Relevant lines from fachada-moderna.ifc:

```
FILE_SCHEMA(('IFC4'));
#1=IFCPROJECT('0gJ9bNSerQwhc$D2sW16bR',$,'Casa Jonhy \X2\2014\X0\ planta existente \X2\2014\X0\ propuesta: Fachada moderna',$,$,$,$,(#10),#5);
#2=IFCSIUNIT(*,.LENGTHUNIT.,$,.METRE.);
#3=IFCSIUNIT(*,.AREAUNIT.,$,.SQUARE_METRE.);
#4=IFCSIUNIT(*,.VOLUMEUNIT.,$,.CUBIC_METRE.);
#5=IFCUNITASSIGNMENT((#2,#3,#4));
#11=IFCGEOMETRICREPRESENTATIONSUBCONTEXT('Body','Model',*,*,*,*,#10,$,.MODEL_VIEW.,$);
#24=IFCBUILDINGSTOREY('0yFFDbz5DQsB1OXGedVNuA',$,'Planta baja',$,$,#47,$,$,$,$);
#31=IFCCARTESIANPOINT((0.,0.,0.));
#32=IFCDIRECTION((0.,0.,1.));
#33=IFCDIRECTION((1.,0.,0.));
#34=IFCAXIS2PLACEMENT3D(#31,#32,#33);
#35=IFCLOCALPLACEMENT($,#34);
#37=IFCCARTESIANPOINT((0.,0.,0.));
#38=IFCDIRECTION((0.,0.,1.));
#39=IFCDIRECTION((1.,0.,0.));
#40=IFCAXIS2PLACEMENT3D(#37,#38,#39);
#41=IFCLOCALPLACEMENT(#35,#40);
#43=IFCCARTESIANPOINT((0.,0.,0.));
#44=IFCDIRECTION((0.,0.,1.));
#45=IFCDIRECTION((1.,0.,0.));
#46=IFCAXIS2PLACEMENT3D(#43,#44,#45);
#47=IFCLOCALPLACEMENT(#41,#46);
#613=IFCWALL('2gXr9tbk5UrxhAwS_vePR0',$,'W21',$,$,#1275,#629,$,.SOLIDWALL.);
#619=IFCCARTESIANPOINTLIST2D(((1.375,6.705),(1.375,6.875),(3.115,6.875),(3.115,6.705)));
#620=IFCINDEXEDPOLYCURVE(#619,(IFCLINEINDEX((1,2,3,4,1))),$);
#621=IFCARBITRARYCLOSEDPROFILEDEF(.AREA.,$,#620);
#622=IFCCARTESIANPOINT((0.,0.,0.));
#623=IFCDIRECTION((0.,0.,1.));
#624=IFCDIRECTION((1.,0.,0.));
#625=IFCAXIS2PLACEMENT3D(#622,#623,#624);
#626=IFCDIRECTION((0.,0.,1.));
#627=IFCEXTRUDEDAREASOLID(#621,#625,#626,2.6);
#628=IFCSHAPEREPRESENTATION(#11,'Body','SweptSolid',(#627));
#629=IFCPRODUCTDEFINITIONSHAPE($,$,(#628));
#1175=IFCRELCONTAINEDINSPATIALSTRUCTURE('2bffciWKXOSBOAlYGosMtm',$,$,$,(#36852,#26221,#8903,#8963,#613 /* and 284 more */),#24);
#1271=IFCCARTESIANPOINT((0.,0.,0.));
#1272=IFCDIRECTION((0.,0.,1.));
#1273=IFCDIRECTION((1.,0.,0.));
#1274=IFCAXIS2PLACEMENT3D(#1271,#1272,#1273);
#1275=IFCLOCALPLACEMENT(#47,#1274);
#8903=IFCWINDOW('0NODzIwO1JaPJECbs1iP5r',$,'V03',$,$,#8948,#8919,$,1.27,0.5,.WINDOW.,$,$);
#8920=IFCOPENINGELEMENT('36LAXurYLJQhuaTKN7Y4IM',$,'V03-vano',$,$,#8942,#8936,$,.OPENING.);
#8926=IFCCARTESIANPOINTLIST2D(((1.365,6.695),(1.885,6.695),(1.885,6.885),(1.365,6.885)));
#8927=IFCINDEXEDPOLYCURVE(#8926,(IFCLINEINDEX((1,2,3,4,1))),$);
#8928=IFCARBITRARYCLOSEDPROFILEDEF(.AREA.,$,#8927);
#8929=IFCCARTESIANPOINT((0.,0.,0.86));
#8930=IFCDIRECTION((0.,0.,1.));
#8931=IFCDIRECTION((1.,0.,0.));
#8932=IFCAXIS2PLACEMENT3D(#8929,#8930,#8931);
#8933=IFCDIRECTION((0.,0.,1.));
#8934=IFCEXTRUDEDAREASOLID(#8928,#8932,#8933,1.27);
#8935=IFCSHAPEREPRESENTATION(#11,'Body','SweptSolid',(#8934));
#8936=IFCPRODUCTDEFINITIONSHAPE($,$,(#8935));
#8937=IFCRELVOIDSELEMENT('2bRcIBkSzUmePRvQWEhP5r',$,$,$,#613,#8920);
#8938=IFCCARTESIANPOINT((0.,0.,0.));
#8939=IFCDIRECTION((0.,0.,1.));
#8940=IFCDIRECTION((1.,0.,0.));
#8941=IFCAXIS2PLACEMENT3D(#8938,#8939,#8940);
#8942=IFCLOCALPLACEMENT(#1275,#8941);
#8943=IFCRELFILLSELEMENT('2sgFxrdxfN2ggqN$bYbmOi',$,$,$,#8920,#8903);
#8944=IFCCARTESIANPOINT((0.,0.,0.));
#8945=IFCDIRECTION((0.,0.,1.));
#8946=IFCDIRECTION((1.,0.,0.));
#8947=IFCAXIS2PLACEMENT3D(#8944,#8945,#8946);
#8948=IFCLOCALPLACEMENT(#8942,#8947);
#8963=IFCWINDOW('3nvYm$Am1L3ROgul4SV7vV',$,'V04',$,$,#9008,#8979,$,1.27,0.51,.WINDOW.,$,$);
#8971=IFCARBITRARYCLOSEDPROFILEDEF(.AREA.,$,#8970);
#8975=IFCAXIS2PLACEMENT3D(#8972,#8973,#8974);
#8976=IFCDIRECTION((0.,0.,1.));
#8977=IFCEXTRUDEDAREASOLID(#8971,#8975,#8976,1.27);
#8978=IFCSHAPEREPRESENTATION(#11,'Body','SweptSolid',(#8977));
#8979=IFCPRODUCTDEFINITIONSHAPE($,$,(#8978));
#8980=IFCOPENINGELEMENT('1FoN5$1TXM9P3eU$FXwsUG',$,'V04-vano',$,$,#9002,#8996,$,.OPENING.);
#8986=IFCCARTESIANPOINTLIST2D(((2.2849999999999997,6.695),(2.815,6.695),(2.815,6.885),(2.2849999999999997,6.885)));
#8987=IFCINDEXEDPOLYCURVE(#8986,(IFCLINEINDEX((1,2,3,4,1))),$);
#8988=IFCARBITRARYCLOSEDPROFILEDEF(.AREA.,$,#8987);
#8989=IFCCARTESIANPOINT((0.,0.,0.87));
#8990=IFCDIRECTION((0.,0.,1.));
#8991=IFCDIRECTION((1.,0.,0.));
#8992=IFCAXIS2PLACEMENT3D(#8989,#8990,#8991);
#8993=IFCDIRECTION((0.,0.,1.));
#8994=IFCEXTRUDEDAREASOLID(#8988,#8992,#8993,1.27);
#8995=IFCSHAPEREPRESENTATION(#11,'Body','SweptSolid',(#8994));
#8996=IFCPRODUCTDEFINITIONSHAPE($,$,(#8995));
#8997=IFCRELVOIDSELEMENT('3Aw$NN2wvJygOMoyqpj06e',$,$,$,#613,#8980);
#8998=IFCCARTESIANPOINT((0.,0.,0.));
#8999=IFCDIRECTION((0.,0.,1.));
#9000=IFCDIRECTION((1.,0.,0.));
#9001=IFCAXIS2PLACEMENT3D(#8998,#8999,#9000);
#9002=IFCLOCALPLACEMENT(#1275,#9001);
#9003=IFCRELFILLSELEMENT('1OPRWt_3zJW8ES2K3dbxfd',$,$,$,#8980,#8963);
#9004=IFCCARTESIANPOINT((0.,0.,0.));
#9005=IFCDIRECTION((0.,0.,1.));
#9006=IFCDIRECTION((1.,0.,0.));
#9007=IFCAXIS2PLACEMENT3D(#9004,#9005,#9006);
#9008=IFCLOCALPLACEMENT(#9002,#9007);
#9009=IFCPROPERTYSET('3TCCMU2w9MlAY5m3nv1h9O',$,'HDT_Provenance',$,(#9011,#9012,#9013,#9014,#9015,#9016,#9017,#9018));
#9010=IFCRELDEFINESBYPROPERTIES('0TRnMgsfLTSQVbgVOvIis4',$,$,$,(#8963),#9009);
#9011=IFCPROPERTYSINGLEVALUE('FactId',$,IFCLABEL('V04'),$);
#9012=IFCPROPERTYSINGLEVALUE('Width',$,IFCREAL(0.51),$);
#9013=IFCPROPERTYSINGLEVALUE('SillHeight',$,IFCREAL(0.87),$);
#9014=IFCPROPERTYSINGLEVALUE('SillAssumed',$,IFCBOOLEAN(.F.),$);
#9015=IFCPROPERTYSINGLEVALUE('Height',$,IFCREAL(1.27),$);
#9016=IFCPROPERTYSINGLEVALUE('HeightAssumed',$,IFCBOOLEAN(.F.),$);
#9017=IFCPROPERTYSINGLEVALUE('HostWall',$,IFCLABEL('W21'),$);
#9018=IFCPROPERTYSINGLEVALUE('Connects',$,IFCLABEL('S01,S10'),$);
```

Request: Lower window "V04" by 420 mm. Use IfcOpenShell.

```python
import numpy as np
import ifcopenshell
import ifcopenshell.api.geometry
import ifcopenshell.api.pset
import ifcopenshell.util.element
import ifcopenshell.util.placement
import ifcopenshell.util.unit

model = ifcopenshell.open("fachada-moderna.ifc")
unit_scale = ifcopenshell.util.unit.calculate_unit_scale(model)

window = model.by_id(8963)
opening = window.FillsVoids[0].RelatingOpeningElement
dz = -0.42

shift = np.array([0.0, 0.0, dz])
# The window is placed relative to its opening, so it follows when the opening moves.
matrix = ifcopenshell.util.placement.get_local_placement(opening.ObjectPlacement)
matrix[:3, 3] += shift
ifcopenshell.api.geometry.edit_object_placement(
    model, product=opening, matrix=matrix, is_si=False, should_transform_children=True
)

# Keep the stored heights in step.
pset = model.by_id(ifcopenshell.util.element.get_pset(window, "HDT_Provenance", should_inherit=False)["id"])
ifcopenshell.api.pset.edit_pset(model, pset=pset, properties={
    "SillHeight": model.create_entity("IfcReal", ifcopenshell.util.element.get_pset(window, "HDT_Provenance", "SillHeight") + dz),
})

print(f"moved by {dz * unit_scale:+.3f} m")

model.write("fachada-moderna_v2.ifc")
```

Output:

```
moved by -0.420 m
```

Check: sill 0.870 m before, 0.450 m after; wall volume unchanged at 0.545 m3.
